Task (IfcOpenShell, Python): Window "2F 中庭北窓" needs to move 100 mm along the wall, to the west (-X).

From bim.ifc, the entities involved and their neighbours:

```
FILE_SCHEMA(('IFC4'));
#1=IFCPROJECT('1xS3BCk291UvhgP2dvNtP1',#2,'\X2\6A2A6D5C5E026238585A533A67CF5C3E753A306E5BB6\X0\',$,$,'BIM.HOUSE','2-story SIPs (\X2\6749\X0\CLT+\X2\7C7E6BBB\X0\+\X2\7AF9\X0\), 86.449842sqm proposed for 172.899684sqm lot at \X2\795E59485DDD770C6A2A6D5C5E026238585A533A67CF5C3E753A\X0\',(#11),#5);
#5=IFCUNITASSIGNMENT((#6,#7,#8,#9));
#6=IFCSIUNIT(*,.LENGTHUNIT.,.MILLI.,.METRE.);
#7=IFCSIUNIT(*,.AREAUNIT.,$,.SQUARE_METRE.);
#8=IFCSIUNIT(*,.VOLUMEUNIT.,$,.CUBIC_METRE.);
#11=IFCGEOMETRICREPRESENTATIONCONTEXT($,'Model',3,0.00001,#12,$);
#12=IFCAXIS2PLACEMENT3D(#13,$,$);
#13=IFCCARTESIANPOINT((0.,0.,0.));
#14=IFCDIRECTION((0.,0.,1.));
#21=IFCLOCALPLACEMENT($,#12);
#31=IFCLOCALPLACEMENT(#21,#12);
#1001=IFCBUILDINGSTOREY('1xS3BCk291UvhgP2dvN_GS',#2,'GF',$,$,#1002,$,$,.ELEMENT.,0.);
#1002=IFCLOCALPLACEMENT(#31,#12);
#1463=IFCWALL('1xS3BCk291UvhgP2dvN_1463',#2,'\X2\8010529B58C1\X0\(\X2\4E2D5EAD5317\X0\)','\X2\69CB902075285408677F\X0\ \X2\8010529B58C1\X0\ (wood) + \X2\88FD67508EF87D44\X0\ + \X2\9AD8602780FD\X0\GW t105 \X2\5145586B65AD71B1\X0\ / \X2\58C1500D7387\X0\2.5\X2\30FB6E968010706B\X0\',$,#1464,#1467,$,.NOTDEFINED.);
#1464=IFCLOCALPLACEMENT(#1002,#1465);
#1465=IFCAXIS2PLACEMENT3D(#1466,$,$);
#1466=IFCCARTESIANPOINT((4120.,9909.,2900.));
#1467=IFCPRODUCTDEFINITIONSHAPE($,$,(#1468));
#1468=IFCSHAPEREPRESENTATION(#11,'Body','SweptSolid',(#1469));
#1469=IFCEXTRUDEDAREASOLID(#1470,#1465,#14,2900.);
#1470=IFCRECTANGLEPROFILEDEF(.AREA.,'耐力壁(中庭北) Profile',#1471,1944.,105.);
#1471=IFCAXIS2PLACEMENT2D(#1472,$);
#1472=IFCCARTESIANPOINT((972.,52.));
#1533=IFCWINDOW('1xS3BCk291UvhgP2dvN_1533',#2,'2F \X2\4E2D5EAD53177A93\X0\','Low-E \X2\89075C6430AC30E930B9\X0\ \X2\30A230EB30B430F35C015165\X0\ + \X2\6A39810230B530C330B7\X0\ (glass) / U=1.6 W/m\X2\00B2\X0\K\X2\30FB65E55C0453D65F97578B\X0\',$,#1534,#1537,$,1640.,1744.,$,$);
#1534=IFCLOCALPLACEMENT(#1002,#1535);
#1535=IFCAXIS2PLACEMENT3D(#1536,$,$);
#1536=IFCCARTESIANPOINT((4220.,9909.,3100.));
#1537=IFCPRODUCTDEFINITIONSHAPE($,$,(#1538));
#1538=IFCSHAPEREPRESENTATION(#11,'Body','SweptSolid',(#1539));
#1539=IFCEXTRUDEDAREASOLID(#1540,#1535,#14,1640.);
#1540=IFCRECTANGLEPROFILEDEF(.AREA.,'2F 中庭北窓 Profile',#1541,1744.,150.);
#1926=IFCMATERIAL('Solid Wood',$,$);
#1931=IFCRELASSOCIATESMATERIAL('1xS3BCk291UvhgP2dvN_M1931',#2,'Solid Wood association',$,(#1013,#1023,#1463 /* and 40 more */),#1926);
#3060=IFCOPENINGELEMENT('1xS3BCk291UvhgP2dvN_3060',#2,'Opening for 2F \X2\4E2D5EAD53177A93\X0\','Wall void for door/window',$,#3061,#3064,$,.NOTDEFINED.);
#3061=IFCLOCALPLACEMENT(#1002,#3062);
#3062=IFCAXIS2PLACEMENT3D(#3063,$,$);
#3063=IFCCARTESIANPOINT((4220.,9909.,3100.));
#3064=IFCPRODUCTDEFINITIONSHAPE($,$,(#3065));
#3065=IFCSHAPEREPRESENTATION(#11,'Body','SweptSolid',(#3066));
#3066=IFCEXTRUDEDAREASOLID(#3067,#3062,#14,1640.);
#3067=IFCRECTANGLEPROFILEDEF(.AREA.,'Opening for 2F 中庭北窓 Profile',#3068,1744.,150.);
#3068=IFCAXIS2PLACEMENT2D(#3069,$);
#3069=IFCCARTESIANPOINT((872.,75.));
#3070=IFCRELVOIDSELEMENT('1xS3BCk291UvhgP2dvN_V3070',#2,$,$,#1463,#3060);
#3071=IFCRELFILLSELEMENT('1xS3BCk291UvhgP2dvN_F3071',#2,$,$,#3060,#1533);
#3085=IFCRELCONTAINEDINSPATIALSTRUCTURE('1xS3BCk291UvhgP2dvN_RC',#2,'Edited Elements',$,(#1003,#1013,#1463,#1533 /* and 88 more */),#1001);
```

```python
import ifcopenshell
import ifcopenshell.api.geometry
import ifcopenshell.util.placement
import ifcopenshell.util.unit

model = ifcopenshell.open("bim.ifc")
unit_scale = ifcopenshell.util.unit.calculate_unit_scale(model)

window = model.by_guid("1xS3BCk291UvhgP2dvN_1533")
opening = window.FillsVoids[0].RelatingOpeningElement
wall = opening.VoidsElements[0].RelatingBuildingElement

wall_matrix = ifcopenshell.util.placement.get_local_placement(wall.ObjectPlacement)
shift = wall_matrix[:3, 0] * -0.1 / unit_scale
before = ifcopenshell.util.placement.get_local_placement(window.ObjectPlacement)[:3, 3].copy()

# The window is not placed relative to its opening, so move both.
for product in (opening, window):
    matrix = ifcopenshell.util.placement.get_local_placement(product.ObjectPlacement)
    matrix[:3, 3] += shift
    ifcopenshell.api.geometry.edit_object_placement(model, product=product, matrix=matrix, is_si=False)

after = ifcopenshell.util.placement.get_local_placement(window.ObjectPlacement)[:3, 3]
print("window moved by", (after - before).round(3) + 0.0)

model.write("bim-out.ifc")
```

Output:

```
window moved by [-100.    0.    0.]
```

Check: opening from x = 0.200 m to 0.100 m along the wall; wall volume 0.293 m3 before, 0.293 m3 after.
